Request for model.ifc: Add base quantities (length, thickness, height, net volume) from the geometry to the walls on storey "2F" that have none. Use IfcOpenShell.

First a look at what the model holds.

```python
import ifcopenshell
import ifcopenshell.util.element
import ifcopenshell.util.unit

model = ifcopenshell.open("model.ifc")
print(model.schema)
for unit_type in ("LENGTHUNIT", "AREAUNIT", "VOLUMEUNIT"):
    print(unit_type, ifcopenshell.util.unit.calculate_unit_scale(model, unit_type))
storey = next(s for s in model.by_type("IfcBuildingStorey") if s.Name == "2F")
walls = [e for e in ifcopenshell.util.element.get_decomposition(storey) if e.is_a("IfcWall")]
for e in sorted(walls, key=lambda e: e.id()):
    print(e.id(), e.is_a(), e.Name, list(ifcopenshell.util.element.get_psets(e, qtos_only=True)), sep=" | ")
```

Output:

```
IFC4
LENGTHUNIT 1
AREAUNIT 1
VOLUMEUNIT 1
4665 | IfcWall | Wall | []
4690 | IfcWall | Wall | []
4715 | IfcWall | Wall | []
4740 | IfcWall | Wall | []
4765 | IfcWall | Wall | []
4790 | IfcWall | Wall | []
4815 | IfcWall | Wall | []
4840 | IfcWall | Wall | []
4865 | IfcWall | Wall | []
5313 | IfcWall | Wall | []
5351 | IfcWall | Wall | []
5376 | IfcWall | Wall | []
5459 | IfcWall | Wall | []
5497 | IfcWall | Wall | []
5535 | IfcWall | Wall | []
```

```python
import ifcopenshell
import ifcopenshell.api.pset
import ifcopenshell.geom
import ifcopenshell.util.element
import ifcopenshell.util.shape
import ifcopenshell.util.unit

model = ifcopenshell.open("model.ifc")
unit_scale = ifcopenshell.util.unit.calculate_unit_scale(model)
volume_scale = ifcopenshell.util.unit.calculate_unit_scale(model, "VOLUMEUNIT")
settings = ifcopenshell.geom.settings()

storey = next(s for s in model.by_type("IfcBuildingStorey") if s.Name == "2F")
walls = [e for e in ifcopenshell.util.element.get_decomposition(storey) if e.is_a("IfcWall")]

for e in sorted(walls, key=lambda e: e.id()):
    if ifcopenshell.util.element.get_psets(e, qtos_only=True, should_inherit=False):
        continue
    # Geometry comes back in metres, in the element's own axes.
    shape = ifcopenshell.geom.create_shape(settings, e)
    values = {
        "Length": ifcopenshell.util.shape.get_x(shape.geometry) / unit_scale,
        "Width": ifcopenshell.util.shape.get_y(shape.geometry) / unit_scale,
        "Height": ifcopenshell.util.shape.get_z(shape.geometry) / unit_scale,
        "NetVolume": ifcopenshell.util.shape.get_volume(shape.geometry) / volume_scale,
    }
    qto = ifcopenshell.api.pset.add_qto(model, product=e, name="Qto_WallBaseQuantities")
    ifcopenshell.api.pset.edit_qto(model, qto=qto, properties=values)
    print(e.id(), {k: round(v, 3) for k, v in values.items()})

model.write("model_rev.ifc")
```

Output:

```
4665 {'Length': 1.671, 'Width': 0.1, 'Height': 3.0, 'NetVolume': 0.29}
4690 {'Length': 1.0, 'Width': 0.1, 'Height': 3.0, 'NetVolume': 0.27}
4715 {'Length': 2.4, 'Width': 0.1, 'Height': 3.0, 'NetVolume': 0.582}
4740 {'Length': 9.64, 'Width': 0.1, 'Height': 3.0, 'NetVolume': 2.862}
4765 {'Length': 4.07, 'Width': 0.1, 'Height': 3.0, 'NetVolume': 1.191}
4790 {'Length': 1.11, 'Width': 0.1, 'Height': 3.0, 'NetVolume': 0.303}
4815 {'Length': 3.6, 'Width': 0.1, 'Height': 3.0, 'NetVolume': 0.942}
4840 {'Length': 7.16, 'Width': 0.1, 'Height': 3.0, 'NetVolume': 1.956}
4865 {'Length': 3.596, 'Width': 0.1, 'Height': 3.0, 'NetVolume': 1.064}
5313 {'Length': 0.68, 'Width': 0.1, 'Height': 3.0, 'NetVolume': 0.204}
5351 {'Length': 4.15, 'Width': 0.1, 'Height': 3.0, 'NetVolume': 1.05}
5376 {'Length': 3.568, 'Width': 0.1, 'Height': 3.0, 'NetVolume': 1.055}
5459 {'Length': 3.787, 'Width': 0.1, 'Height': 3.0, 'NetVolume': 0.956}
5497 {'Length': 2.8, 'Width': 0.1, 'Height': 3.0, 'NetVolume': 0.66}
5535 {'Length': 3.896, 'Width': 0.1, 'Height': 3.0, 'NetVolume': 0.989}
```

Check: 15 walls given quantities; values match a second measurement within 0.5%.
